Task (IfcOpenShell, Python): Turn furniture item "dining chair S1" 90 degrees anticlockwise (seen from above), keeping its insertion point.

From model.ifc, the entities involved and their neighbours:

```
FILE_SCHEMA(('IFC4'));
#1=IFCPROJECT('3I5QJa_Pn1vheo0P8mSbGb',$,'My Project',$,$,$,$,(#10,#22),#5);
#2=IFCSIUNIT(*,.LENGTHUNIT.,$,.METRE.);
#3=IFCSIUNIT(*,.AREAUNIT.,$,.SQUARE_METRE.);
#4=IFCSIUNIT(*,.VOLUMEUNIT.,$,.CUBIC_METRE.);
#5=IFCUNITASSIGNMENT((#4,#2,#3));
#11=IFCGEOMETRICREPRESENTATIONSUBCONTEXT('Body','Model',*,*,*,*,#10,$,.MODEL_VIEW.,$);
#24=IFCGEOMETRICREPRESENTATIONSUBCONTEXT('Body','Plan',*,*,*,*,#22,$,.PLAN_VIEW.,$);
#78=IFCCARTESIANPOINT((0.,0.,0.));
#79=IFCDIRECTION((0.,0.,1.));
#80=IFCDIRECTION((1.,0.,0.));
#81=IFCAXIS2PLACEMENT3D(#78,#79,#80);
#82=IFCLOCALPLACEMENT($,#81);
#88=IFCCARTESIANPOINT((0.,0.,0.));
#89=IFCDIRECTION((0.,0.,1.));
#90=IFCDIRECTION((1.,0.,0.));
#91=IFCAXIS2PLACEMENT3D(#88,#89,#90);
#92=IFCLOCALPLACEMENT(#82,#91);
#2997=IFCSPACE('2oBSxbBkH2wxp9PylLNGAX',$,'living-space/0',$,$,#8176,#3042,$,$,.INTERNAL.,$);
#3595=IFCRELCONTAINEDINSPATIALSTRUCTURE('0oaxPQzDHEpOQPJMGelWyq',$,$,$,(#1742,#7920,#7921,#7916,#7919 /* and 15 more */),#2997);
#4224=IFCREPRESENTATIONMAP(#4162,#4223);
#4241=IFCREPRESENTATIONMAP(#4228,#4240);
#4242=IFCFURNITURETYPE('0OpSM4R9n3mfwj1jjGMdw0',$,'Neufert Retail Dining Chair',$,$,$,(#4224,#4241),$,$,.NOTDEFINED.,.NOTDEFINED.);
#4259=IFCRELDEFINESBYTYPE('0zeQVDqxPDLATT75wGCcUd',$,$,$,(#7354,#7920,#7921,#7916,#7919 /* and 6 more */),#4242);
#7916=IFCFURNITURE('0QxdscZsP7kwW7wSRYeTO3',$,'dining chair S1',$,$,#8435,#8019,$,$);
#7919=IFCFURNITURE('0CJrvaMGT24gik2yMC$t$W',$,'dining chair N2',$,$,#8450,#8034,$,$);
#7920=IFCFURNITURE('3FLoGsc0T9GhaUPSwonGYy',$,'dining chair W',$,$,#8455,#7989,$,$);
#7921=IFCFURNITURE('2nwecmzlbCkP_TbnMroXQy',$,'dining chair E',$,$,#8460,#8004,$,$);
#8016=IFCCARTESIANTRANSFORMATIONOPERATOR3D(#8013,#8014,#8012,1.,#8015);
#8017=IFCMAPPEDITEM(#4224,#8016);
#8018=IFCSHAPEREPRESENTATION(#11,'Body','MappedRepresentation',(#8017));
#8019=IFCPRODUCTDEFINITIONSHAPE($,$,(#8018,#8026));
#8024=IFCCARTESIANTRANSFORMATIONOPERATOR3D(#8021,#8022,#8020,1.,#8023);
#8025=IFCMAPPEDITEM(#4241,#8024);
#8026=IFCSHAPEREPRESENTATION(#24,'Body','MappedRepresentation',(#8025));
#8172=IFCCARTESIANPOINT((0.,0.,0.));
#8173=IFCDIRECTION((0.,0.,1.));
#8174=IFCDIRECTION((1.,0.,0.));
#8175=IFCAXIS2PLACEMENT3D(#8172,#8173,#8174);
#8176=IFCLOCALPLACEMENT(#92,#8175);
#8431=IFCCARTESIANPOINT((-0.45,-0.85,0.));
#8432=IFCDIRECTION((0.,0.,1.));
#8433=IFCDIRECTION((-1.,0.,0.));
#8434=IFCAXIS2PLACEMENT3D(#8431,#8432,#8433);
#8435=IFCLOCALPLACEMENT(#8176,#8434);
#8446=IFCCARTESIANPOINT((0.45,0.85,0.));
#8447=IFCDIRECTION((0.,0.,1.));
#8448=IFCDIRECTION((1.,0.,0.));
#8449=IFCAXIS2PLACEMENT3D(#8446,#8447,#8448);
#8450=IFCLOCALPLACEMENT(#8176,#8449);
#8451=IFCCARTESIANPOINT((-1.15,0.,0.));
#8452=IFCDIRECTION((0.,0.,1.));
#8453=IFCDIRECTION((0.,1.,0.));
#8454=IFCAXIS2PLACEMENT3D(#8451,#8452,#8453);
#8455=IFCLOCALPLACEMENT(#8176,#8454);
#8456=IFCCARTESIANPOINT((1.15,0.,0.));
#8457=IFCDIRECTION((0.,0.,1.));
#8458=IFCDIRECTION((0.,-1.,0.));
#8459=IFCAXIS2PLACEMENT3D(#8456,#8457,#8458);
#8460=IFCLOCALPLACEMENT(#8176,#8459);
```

```python
import ifcopenshell
import ifcopenshell.api.geometry
import ifcopenshell.util.placement

model = ifcopenshell.open("model.ifc")

item = model.by_id(7916)
matrix = ifcopenshell.util.placement.get_local_placement(item.ObjectPlacement)
matrix = matrix @ ifcopenshell.util.placement.rotation(90, "Z")
ifcopenshell.api.geometry.edit_object_placement(model, product=item, matrix=matrix, is_si=False)

print(ifcopenshell.util.placement.get_local_placement(item.ObjectPlacement).round(3) + 0.0)

model.write("model-out.ifc")
```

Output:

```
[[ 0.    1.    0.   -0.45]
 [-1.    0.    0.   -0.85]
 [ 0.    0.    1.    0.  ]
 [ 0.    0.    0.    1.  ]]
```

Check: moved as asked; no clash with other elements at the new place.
